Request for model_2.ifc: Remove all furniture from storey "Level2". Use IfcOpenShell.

First a look at what the model holds.

```python
import ifcopenshell
import ifcopenshell.util.element

model = ifcopenshell.open("model_2.ifc")
print(model.schema)
storey = next(s for s in model.by_type("IfcBuildingStorey") if s.Name == "Level2")
furniture = [e for e in ifcopenshell.util.element.get_decomposition(storey) if e.is_a("IfcFurnishingElement")]
seen = {}
for e in furniture:
    element_type = ifcopenshell.util.element.get_type(e)
    name = element_type.Name if element_type not in (None, e) else None
    seen[name] = seen.get(name, 0) + 1
for name, count in sorted(seen.items(), key=str):
    print(count, "x", name)
```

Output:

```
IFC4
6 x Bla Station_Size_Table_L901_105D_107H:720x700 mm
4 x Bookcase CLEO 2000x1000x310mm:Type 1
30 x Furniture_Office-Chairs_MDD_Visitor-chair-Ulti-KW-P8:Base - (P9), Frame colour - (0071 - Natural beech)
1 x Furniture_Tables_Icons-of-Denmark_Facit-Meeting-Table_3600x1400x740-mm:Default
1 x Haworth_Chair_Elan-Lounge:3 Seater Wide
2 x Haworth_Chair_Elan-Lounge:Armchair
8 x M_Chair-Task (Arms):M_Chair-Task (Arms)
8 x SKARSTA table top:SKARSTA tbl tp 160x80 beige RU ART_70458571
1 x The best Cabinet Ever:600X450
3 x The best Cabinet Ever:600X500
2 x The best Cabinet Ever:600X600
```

```python
import ifcopenshell
import ifcopenshell.api.root
import ifcopenshell.util.element

model = ifcopenshell.open("model_2.ifc")

storey = next(s for s in model.by_type("IfcBuildingStorey") if s.Name == "Level2")
furniture = [e for e in ifcopenshell.util.element.get_decomposition(storey) if e.is_a("IfcFurnishingElement")]

for e in furniture:
    ifcopenshell.api.root.remove_product(model, product=e)
print(len(furniture), "removed")

model.write("model_2-out.ifc")
```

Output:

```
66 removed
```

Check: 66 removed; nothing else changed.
